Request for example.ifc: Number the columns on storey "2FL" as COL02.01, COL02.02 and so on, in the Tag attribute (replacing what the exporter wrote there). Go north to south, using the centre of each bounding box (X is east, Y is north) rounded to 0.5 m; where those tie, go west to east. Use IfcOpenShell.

First a look at what the model holds.

```python
import ifcopenshell
import ifcopenshell.util.element
import ifcopenshell.util.placement

model = ifcopenshell.open("example.ifc")
print(model.schema)
storey = next(s for s in model.by_type("IfcBuildingStorey") if s.Name == "2FL")
columns = [e for e in ifcopenshell.util.element.get_decomposition(storey) if e.is_a("IfcColumn")]
for e in sorted(columns, key=lambda e: e.id()):
    origin = ifcopenshell.util.placement.get_local_placement(e.ObjectPlacement)[:3, 3]
    print(e.id(), e.Tag, e.Name, origin.round(2) + 0.0, sep=" | ")
```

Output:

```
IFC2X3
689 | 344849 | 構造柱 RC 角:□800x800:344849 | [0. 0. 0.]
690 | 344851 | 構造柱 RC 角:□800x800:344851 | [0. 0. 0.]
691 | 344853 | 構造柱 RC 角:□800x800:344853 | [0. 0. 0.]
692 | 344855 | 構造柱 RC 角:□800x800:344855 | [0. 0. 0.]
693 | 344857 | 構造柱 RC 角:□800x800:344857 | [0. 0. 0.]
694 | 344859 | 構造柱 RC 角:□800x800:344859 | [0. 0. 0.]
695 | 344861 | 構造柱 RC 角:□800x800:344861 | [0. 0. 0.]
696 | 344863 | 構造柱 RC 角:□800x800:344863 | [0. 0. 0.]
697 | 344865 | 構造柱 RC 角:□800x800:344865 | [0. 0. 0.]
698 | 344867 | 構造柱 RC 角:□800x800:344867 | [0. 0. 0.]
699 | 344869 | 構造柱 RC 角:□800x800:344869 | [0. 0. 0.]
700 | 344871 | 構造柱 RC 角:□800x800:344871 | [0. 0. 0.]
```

```python
import ifcopenshell
import ifcopenshell.geom
import ifcopenshell.util.element
import ifcopenshell.util.shape

model = ifcopenshell.open("example.ifc")
settings = ifcopenshell.geom.settings()
settings.set("use-world-coords", True)


def centre(element):
    shape = ifcopenshell.geom.create_shape(settings, element)
    return ifcopenshell.util.shape.get_bbox_centroid(shape.geometry)


storey = next(s for s in model.by_type("IfcBuildingStorey") if s.Name == "2FL")
columns = [e for e in ifcopenshell.util.element.get_decomposition(storey) if e.is_a("IfcColumn")]

# Insertion points can sit at a corner or the storey origin, so sort by the geometry (in metres).
centres = {e: centre(e) for e in columns}
columns.sort(key=lambda e: (-round(centres[e][1] / 0.5), centres[e][0]))

for i, e in enumerate(columns, start=1):
    number = f"COL02.{i:02d}"
    e.Tag = number
    print(e.id(), number)

model.write("example-out.ifc")
```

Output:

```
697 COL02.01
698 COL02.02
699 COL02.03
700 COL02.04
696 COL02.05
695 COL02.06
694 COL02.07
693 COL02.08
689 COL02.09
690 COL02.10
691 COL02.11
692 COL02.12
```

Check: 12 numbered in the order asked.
